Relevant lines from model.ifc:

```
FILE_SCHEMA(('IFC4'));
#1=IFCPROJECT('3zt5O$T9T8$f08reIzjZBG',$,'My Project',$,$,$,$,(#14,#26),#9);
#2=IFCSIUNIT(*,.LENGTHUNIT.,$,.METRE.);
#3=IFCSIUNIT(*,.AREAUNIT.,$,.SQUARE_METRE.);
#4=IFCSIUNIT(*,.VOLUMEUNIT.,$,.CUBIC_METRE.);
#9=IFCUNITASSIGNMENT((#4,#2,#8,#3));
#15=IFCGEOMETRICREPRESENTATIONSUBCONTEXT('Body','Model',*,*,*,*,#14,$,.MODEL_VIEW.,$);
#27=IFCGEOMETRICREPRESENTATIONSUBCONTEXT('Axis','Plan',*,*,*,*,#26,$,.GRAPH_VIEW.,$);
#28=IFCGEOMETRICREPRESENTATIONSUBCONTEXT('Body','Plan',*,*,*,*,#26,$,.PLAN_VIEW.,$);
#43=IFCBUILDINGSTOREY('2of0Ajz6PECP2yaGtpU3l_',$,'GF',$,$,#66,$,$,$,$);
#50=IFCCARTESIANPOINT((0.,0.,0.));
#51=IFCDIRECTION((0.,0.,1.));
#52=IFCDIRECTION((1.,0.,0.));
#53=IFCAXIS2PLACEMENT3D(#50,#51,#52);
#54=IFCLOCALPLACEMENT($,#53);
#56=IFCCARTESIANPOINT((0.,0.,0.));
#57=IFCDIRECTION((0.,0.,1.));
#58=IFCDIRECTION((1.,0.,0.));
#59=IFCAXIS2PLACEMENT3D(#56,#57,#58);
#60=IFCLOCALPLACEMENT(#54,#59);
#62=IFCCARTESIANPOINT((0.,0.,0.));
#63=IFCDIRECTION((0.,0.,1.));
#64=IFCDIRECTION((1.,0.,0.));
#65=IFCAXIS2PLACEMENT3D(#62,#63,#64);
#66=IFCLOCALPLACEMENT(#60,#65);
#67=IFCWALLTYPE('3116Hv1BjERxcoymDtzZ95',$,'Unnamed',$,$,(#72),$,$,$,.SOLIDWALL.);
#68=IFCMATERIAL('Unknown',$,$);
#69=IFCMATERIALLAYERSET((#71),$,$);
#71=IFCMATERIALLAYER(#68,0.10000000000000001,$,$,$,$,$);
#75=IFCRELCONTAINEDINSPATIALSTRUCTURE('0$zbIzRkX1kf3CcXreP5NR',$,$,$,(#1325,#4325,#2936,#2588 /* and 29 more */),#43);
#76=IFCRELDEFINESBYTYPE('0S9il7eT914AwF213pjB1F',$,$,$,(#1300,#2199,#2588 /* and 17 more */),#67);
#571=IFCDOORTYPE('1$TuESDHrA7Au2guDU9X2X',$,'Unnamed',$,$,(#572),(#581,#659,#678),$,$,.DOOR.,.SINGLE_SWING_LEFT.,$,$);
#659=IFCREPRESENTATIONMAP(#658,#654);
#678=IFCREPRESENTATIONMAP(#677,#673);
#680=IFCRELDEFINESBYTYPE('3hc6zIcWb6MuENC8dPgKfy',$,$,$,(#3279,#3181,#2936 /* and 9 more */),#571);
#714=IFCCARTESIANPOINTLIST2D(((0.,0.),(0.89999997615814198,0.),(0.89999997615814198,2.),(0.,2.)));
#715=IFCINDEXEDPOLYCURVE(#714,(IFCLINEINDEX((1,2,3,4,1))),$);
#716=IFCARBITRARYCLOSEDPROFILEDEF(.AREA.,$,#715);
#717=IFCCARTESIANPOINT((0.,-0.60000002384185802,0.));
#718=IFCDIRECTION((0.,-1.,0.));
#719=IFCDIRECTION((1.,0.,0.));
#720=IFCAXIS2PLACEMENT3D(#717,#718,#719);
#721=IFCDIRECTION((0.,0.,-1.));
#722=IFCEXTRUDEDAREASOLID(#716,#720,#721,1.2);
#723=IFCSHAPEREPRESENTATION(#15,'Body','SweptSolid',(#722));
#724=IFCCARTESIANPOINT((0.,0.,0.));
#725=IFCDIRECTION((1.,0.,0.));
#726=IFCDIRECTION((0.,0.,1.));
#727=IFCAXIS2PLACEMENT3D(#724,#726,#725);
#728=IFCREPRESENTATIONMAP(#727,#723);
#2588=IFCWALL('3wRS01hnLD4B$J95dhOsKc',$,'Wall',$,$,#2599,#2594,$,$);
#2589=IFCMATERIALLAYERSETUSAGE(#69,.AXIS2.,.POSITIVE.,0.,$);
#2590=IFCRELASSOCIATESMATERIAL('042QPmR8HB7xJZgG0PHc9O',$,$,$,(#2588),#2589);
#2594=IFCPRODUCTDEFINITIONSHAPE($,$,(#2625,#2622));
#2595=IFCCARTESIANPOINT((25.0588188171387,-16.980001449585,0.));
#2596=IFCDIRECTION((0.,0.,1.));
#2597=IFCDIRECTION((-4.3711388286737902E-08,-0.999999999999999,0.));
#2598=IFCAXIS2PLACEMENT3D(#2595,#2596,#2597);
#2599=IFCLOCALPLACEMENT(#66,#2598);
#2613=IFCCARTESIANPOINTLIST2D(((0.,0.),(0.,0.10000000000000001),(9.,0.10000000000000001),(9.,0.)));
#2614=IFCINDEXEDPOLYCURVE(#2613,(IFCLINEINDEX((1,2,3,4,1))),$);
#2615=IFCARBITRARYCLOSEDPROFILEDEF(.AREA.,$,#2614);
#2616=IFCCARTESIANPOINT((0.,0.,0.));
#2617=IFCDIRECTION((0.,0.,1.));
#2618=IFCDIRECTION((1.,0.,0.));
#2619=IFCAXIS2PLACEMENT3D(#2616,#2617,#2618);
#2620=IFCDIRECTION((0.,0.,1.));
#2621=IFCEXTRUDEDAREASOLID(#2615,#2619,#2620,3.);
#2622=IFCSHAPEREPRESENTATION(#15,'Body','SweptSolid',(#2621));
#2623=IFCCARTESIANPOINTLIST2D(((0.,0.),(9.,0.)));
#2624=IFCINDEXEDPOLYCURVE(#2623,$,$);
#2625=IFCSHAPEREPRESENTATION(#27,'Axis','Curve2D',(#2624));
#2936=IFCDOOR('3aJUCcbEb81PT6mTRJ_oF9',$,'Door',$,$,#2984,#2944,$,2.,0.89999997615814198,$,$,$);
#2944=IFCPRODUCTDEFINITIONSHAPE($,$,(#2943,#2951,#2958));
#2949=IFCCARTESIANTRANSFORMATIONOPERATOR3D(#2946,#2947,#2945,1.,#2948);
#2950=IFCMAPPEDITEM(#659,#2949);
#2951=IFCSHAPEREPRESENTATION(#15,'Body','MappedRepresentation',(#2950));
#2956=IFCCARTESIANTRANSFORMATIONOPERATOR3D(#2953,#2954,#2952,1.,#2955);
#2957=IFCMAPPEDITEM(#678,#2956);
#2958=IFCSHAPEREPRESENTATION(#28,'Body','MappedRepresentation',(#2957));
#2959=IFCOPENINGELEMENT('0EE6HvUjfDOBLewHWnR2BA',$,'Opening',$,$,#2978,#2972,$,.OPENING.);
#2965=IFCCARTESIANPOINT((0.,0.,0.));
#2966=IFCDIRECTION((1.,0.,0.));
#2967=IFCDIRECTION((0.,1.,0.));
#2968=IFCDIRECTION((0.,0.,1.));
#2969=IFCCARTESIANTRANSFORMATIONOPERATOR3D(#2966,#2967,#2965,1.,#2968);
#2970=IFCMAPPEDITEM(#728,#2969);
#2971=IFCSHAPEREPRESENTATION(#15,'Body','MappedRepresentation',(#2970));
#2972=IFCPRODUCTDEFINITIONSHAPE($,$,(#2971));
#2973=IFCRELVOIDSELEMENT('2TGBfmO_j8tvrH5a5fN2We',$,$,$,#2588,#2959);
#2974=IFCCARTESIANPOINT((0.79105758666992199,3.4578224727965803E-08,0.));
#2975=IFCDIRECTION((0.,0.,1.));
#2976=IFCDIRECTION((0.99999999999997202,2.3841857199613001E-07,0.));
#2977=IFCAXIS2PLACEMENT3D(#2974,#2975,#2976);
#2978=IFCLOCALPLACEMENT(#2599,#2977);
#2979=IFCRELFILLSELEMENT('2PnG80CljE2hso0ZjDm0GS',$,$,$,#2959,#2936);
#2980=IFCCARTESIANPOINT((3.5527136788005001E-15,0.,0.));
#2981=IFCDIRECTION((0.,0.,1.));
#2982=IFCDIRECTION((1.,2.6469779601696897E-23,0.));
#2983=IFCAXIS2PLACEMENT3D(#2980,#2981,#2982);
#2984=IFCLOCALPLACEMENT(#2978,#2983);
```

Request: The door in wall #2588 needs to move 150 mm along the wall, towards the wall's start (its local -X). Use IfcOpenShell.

```python
import ifcopenshell
import ifcopenshell.api.geometry
import ifcopenshell.util.placement
import ifcopenshell.util.unit

model = ifcopenshell.open("model.ifc")
unit_scale = ifcopenshell.util.unit.calculate_unit_scale(model)

door = model.by_guid("3aJUCcbEb81PT6mTRJ_oF9")
opening = door.FillsVoids[0].RelatingOpeningElement
wall = opening.VoidsElements[0].RelatingBuildingElement

wall_matrix = ifcopenshell.util.placement.get_local_placement(wall.ObjectPlacement)
shift = wall_matrix[:3, 0] * -0.15 / unit_scale
before = ifcopenshell.util.placement.get_local_placement(door.ObjectPlacement)[:3, 3].copy()

# The door is placed relative to its opening, so it follows when the opening moves.
matrix = ifcopenshell.util.placement.get_local_placement(opening.ObjectPlacement)
matrix[:3, 3] += shift
ifcopenshell.api.geometry.edit_object_placement(
    model, product=opening, matrix=matrix, is_si=False, should_transform_children=True
)

after = ifcopenshell.util.placement.get_local_placement(door.ObjectPlacement)[:3, 3]
print("door moved by", (after - before).round(3) + 0.0)

model.write("model_updated.ifc")
```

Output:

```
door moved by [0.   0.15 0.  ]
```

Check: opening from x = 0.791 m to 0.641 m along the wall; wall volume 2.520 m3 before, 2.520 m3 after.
